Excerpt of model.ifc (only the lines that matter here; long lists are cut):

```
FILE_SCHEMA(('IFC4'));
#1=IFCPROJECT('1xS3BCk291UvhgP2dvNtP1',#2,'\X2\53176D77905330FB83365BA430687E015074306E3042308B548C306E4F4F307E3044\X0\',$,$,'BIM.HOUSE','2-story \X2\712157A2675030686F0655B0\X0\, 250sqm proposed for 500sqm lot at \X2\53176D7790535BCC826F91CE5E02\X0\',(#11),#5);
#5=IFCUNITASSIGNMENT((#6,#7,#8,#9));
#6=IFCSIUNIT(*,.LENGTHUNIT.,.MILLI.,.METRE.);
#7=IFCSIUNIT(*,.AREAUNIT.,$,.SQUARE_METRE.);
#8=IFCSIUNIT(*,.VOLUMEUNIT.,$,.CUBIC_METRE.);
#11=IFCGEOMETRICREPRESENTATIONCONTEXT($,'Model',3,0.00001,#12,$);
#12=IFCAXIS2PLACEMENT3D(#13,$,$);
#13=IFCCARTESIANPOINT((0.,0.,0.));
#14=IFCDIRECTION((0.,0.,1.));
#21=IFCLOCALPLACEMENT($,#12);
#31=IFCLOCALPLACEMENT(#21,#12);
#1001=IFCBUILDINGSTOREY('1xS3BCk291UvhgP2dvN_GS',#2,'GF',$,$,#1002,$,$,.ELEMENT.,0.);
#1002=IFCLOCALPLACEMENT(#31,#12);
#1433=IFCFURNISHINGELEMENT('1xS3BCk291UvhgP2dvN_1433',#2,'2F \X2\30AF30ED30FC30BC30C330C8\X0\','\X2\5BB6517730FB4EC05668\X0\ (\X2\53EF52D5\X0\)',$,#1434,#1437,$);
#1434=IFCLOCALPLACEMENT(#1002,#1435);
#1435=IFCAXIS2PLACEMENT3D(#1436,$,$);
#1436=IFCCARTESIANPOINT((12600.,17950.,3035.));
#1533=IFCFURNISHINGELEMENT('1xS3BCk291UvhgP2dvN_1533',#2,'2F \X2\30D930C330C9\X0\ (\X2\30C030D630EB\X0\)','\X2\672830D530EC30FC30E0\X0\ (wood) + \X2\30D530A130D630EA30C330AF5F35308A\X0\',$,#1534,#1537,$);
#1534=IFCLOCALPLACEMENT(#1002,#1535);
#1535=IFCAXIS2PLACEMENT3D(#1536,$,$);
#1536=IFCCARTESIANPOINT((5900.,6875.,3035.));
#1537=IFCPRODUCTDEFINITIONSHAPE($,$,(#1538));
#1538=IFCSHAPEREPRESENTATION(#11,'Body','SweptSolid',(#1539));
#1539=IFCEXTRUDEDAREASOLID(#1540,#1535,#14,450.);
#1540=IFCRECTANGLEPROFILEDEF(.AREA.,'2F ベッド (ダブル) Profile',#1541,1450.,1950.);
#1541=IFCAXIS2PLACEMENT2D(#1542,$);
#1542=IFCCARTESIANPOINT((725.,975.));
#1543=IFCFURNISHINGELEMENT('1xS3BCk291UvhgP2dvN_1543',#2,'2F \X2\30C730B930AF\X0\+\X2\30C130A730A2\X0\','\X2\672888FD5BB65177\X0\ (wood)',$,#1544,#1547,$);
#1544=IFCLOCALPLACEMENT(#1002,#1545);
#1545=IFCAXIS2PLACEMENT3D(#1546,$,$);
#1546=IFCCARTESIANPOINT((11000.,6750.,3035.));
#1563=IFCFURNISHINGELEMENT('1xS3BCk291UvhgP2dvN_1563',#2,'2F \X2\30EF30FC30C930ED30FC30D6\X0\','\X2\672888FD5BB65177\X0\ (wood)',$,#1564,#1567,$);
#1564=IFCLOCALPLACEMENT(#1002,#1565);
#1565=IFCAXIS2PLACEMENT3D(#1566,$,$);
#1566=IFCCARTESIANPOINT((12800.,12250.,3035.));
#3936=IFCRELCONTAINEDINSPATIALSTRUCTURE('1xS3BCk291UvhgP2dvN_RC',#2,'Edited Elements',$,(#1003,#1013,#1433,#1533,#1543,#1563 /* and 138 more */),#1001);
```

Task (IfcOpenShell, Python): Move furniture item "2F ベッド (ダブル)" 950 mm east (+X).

```python
import ifcopenshell
import ifcopenshell.api.geometry
import ifcopenshell.util.placement

model = ifcopenshell.open("model.ifc")

item = model.by_guid("1xS3BCk291UvhgP2dvN_1533")
matrix = ifcopenshell.util.placement.get_local_placement(item.ObjectPlacement)
matrix[0, 3] += 950.0
ifcopenshell.api.geometry.edit_object_placement(model, product=item, matrix=matrix, is_si=False)

print(ifcopenshell.util.placement.get_local_placement(item.ObjectPlacement).round(3) + 0.0)

model.write("model_rev.ifc")
```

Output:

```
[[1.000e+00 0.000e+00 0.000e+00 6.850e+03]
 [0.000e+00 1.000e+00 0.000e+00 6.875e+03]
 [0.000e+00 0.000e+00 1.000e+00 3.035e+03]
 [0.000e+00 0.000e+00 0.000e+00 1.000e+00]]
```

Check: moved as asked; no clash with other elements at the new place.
